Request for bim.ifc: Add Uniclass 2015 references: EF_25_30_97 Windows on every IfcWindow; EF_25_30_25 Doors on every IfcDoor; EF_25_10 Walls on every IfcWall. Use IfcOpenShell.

First a look at what the model holds.

```python
import ifcopenshell

model = ifcopenshell.open("bim.ifc")
print(model.schema)
print("classifications:", [c.Name for c in model.by_type("IfcClassification")])
for ifc_class in ("IfcDoor", "IfcRoof", "IfcStair", "IfcWall", "IfcWindow"):
    print(ifc_class, len(model.by_type(ifc_class)))
```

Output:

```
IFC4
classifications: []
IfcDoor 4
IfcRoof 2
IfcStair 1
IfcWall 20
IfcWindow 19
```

```python
import ifcopenshell
import ifcopenshell.api.classification

model = ifcopenshell.open("bim.ifc")

system = ifcopenshell.api.classification.add_classification(model, classification="Uniclass 2015")

codes = {
    "IfcWindow": ("EF_25_30_97", "Windows"),
    "IfcDoor": ("EF_25_30_25", "Doors"),
    "IfcWall": ("EF_25_10", "Walls"),
}
for ifc_class, (code, name) in codes.items():
    products = model.by_type(ifc_class)
    ifcopenshell.api.classification.add_reference(
        model, products=products, classification=system, identification=code, name=name
    )
    print(code, len(products))

model.write("bim-out.ifc")
```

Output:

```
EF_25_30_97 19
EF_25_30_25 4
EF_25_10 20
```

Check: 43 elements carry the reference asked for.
